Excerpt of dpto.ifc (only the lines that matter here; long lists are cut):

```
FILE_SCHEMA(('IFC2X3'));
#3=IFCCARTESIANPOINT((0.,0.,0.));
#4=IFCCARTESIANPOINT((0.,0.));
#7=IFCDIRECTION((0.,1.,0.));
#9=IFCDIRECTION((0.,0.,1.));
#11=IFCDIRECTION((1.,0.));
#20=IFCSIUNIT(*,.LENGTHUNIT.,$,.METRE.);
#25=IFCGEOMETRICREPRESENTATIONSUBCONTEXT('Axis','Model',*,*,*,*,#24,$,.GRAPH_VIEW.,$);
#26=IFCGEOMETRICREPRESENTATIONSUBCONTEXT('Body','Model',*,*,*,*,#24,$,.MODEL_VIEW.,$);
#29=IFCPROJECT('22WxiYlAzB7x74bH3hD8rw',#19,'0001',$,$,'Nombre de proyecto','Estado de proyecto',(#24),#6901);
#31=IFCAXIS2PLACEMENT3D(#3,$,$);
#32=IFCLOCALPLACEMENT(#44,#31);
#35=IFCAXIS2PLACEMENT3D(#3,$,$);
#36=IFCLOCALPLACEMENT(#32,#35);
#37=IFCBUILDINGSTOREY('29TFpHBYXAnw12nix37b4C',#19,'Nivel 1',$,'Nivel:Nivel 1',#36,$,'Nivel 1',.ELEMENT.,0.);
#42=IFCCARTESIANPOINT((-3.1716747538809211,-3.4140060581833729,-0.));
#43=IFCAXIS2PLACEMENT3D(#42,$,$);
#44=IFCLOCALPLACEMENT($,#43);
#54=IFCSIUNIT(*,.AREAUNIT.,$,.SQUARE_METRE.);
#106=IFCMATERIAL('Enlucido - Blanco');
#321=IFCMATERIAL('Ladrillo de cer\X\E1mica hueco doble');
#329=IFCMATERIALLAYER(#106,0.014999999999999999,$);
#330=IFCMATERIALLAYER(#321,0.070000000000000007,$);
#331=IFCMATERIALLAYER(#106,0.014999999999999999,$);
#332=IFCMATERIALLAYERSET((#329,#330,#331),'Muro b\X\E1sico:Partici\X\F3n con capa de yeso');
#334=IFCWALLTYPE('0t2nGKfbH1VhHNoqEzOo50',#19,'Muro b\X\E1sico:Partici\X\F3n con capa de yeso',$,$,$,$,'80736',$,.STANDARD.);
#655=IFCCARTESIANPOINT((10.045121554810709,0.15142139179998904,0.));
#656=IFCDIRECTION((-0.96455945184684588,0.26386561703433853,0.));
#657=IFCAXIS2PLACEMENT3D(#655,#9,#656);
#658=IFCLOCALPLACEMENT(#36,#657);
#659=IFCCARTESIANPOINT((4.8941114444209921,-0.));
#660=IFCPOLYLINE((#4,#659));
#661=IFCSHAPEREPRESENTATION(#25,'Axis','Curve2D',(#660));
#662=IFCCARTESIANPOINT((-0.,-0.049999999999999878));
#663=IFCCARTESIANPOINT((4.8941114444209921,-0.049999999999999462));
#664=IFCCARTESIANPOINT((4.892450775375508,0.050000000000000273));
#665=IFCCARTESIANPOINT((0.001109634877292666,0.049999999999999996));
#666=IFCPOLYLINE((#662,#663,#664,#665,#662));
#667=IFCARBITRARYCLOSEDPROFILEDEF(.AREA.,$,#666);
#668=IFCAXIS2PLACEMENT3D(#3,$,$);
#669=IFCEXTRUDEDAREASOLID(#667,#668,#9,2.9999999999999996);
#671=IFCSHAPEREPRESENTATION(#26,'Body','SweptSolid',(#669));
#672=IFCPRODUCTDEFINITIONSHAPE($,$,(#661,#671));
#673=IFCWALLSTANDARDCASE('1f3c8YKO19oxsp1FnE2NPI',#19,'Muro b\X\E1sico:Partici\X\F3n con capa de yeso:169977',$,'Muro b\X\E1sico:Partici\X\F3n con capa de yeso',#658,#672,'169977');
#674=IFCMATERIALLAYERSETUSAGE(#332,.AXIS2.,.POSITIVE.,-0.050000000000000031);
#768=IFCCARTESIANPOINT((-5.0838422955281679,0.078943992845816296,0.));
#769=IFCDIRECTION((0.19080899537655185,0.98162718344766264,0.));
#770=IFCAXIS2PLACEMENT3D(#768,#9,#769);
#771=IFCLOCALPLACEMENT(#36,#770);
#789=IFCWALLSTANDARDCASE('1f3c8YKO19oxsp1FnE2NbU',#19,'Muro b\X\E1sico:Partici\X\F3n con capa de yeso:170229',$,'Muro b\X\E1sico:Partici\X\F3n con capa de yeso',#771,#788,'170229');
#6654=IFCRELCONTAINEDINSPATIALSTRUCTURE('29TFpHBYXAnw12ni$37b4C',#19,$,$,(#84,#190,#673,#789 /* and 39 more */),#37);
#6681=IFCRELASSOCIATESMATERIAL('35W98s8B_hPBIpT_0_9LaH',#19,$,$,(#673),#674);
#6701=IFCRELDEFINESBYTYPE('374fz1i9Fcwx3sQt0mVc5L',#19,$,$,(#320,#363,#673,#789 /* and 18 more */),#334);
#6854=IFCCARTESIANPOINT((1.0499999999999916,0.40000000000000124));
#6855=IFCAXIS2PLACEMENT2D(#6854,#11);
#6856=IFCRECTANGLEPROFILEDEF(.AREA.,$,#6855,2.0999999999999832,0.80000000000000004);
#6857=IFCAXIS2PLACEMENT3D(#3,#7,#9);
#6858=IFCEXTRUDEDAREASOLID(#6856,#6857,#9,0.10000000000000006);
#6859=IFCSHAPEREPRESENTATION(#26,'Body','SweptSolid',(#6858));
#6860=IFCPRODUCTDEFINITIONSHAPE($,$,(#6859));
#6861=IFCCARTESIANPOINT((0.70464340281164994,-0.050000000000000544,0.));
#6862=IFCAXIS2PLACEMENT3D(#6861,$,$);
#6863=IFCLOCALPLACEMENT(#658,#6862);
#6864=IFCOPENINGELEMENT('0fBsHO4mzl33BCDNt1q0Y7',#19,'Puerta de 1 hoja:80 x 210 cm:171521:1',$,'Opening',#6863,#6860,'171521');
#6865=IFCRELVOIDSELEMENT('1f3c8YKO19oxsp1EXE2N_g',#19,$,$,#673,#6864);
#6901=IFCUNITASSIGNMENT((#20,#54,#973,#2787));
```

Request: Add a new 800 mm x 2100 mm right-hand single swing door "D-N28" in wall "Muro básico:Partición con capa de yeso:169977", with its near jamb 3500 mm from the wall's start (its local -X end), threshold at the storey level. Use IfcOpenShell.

```python
import numpy as np
import ifcopenshell
import ifcopenshell.api.feature
import ifcopenshell.api.geometry
import ifcopenshell.api.root
import ifcopenshell.api.spatial
import ifcopenshell.api.type
import ifcopenshell.geom
import ifcopenshell.util.element
import ifcopenshell.util.placement
import ifcopenshell.util.representation
import ifcopenshell.util.shape
import ifcopenshell.util.unit

model = ifcopenshell.open("dpto.ifc")
unit_scale = ifcopenshell.util.unit.calculate_unit_scale(model)
settings = ifcopenshell.geom.settings()


def volume(element):
    """Net volume in cubic metres, openings subtracted."""
    shape = ifcopenshell.geom.create_shape(settings, element)
    return ifcopenshell.util.shape.get_volume(shape.geometry)


wall = model.by_guid("1f3c8YKO19oxsp1FnE2NPI")
storey = ifcopenshell.util.element.get_container(wall, ifc_class="IfcBuildingStorey")
context = ifcopenshell.util.representation.get_context(model, "Model", "Body", "MODEL_VIEW")
before = volume(wall)

width, height, from_end, sill = 0.8, 2.1, 3.5, 0.0  # metres

# The wall runs along its own X axis, and the end named is its -X end.
wall_shape = ifcopenshell.geom.create_shape(settings, wall)
x, y, z = ifcopenshell.util.shape.get_vertices(wall_shape.geometry).T
start = x.min() + from_end
face, thickness = float(y.min()), float(y.max() - y.min())
wall_matrix = ifcopenshell.util.placement.get_local_placement(wall.ObjectPlacement)
level = ifcopenshell.util.placement.get_local_placement(storey.ObjectPlacement)[2, 3]


def in_wall(x, y):
    """Placement at x, y metres in the wall's axes, at sill height."""
    matrix = wall_matrix.copy()
    matrix[:, 3] = wall_matrix @ np.array([x / unit_scale, y / unit_scale, 0.0, 1.0])
    matrix[2, 3] = level + sill / unit_scale
    return matrix


# Opening: a box that overshoots both wall faces by 50 mm.
opening = ifcopenshell.api.root.create_entity(model, ifc_class="IfcOpeningElement")
box = ifcopenshell.api.geometry.add_wall_representation(
    model, context=context, length=width, height=height, thickness=thickness + 0.1
)
ifcopenshell.api.geometry.assign_representation(model, product=opening, representation=box)
ifcopenshell.api.geometry.edit_object_placement(model, product=opening, matrix=in_wall(start, face - 0.05), is_si=False)
ifcopenshell.api.feature.add_feature(model, feature=opening, element=wall)

door = ifcopenshell.api.root.create_entity(model, ifc_class="IfcDoor", name="D-N28")
door.OverallWidth, door.OverallHeight = width / unit_scale, height / unit_scale
body = ifcopenshell.api.geometry.add_door_representation(
    model,
    context=context,
    overall_width=door.OverallWidth,
    overall_height=door.OverallHeight,
    operation_type="SINGLE_SWING_RIGHT",
    lining_properties={"LiningDepth": thickness / unit_scale, "ThresholdDepth": thickness / unit_scale},
)
ifcopenshell.api.geometry.assign_representation(model, product=door, representation=body)
ifcopenshell.api.spatial.assign_container(model, products=[door], relating_structure=storey)
fills = ifcopenshell.api.feature.add_filling(model, opening=opening, element=door)
fills.OwnerHistory = door.OwnerHistory  # required in IFC2X3

# IFC2X3 keeps the operation on the door style.
style = ifcopenshell.api.root.create_entity(model, ifc_class="IfcDoorStyle", name="D-N28")
style.OperationType, style.ConstructionType = "SINGLE_SWING_RIGHT", "NOTDEFINED"
style.ParameterTakesPrecedence = style.Sizeable = False
ifcopenshell.api.type.assign_type(model, related_objects=[door], relating_type=style)

# The lining spans the wall, so the door starts at the wall face.
ifcopenshell.api.geometry.edit_object_placement(model, product=door, matrix=in_wall(start, face), is_si=False)

after = volume(wall)

print(f"wall volume {before:.3f} -> {after:.3f} m3")

model.write("dpto_edited.ifc")
```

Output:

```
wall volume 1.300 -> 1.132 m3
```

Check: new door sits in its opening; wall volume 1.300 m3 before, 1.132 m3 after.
